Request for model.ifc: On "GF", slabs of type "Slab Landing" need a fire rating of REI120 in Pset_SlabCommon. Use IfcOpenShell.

First a look at what the model holds.

```python
import ifcopenshell
import ifcopenshell.util.element

model = ifcopenshell.open("model.ifc")
print(model.schema)
storey = next(s for s in model.by_type("IfcBuildingStorey") if s.Name == "GF")
slabs = [e for e in ifcopenshell.util.element.get_decomposition(storey) if e.is_a("IfcSlab")]
seen = {}
for e in slabs:
    element_type = ifcopenshell.util.element.get_type(e)
    key = (element_type.Name if element_type != e and element_type else None, ifcopenshell.util.element.get_pset(e, "Pset_SlabCommon", "FireRating"))
    seen[key] = seen.get(key, 0) + 1
for (name, value), count in sorted(seen.items(), key=str):
    print(count, "x", name, "|", value)
```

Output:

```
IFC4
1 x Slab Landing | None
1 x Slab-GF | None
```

```python
import ifcopenshell
import ifcopenshell.api.pset
import ifcopenshell.util.element

model = ifcopenshell.open("model.ifc")

storey = next(s for s in model.by_type("IfcBuildingStorey") if s.Name == "GF")
slabs = [e for e in ifcopenshell.util.element.get_decomposition(storey) if e.is_a("IfcSlab")]

count = 0
for e in slabs:
    element_type = ifcopenshell.util.element.get_type(e)
    if element_type in (None, e) or element_type.Name != "Slab Landing":
        continue
    # add_pset returns the element's existing set when there is one.
    pset = ifcopenshell.api.pset.add_pset(model, product=e, name="Pset_SlabCommon")
    ifcopenshell.api.pset.edit_pset(model, pset=pset, properties={"FireRating": "REI120"})
    count += 1

print(count, "slabs updated")

model.write("model-out.ifc")
```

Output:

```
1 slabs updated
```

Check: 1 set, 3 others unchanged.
